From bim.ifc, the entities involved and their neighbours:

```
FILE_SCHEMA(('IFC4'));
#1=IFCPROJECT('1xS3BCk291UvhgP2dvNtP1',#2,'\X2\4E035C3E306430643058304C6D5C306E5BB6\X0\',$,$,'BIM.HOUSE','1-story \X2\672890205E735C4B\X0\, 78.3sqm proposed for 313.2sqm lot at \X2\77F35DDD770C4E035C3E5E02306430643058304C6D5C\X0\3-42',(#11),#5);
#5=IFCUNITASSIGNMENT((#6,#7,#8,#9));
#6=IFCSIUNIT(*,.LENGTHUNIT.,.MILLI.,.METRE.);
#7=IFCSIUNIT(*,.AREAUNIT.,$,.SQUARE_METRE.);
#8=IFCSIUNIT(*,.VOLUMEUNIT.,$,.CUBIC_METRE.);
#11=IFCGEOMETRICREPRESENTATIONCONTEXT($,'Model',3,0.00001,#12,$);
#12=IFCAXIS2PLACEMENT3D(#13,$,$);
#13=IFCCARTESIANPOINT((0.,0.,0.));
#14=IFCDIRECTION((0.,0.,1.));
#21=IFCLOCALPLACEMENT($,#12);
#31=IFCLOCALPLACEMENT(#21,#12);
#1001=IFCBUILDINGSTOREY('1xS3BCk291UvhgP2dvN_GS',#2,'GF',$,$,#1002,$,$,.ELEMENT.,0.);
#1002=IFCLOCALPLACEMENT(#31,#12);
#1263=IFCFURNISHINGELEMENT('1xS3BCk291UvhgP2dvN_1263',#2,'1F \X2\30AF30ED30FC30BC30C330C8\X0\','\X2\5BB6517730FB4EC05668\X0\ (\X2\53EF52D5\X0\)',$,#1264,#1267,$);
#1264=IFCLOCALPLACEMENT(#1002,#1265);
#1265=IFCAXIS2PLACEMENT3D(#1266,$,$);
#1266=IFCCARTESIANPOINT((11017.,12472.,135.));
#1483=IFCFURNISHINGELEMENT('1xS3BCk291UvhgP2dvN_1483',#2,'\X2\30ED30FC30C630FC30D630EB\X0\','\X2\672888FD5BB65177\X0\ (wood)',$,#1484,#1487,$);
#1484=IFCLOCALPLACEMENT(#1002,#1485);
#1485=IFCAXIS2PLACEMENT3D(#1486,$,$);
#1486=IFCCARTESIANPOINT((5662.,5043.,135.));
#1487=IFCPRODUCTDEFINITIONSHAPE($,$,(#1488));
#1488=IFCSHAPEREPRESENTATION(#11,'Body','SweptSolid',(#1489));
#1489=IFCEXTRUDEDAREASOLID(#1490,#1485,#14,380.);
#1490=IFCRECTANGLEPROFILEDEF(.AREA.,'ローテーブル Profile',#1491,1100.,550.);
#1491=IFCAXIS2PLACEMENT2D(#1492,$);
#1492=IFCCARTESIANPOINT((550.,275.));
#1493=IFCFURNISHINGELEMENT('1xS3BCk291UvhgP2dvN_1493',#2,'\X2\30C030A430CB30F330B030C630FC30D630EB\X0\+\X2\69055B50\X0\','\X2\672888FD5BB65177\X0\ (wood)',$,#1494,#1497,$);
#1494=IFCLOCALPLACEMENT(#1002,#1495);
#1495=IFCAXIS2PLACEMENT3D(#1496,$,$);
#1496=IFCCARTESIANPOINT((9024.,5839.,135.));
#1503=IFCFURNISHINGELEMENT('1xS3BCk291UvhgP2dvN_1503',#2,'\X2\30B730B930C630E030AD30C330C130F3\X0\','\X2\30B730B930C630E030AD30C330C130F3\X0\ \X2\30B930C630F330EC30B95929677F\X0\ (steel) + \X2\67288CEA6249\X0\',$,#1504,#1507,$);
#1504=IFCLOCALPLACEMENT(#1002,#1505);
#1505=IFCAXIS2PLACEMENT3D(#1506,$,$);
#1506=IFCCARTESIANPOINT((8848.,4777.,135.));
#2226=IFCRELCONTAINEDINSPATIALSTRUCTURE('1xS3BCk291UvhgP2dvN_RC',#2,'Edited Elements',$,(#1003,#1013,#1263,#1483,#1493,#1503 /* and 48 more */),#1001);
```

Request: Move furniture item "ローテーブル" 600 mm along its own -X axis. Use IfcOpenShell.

```python
import ifcopenshell
import ifcopenshell.api.geometry
import ifcopenshell.util.placement

model = ifcopenshell.open("bim.ifc")

item = model.by_guid("1xS3BCk291UvhgP2dvN_1483")
matrix = ifcopenshell.util.placement.get_local_placement(item.ObjectPlacement)
matrix[:3, 3] -= matrix[:3, 0] * 600.0
ifcopenshell.api.geometry.edit_object_placement(model, product=item, matrix=matrix, is_si=False)

print(ifcopenshell.util.placement.get_local_placement(item.ObjectPlacement).round(3) + 0.0)

model.write("bim-out.ifc")
```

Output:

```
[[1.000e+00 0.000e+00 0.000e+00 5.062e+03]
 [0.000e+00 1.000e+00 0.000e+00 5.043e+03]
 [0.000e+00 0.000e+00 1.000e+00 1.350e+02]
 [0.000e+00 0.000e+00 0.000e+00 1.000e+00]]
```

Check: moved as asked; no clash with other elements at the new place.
